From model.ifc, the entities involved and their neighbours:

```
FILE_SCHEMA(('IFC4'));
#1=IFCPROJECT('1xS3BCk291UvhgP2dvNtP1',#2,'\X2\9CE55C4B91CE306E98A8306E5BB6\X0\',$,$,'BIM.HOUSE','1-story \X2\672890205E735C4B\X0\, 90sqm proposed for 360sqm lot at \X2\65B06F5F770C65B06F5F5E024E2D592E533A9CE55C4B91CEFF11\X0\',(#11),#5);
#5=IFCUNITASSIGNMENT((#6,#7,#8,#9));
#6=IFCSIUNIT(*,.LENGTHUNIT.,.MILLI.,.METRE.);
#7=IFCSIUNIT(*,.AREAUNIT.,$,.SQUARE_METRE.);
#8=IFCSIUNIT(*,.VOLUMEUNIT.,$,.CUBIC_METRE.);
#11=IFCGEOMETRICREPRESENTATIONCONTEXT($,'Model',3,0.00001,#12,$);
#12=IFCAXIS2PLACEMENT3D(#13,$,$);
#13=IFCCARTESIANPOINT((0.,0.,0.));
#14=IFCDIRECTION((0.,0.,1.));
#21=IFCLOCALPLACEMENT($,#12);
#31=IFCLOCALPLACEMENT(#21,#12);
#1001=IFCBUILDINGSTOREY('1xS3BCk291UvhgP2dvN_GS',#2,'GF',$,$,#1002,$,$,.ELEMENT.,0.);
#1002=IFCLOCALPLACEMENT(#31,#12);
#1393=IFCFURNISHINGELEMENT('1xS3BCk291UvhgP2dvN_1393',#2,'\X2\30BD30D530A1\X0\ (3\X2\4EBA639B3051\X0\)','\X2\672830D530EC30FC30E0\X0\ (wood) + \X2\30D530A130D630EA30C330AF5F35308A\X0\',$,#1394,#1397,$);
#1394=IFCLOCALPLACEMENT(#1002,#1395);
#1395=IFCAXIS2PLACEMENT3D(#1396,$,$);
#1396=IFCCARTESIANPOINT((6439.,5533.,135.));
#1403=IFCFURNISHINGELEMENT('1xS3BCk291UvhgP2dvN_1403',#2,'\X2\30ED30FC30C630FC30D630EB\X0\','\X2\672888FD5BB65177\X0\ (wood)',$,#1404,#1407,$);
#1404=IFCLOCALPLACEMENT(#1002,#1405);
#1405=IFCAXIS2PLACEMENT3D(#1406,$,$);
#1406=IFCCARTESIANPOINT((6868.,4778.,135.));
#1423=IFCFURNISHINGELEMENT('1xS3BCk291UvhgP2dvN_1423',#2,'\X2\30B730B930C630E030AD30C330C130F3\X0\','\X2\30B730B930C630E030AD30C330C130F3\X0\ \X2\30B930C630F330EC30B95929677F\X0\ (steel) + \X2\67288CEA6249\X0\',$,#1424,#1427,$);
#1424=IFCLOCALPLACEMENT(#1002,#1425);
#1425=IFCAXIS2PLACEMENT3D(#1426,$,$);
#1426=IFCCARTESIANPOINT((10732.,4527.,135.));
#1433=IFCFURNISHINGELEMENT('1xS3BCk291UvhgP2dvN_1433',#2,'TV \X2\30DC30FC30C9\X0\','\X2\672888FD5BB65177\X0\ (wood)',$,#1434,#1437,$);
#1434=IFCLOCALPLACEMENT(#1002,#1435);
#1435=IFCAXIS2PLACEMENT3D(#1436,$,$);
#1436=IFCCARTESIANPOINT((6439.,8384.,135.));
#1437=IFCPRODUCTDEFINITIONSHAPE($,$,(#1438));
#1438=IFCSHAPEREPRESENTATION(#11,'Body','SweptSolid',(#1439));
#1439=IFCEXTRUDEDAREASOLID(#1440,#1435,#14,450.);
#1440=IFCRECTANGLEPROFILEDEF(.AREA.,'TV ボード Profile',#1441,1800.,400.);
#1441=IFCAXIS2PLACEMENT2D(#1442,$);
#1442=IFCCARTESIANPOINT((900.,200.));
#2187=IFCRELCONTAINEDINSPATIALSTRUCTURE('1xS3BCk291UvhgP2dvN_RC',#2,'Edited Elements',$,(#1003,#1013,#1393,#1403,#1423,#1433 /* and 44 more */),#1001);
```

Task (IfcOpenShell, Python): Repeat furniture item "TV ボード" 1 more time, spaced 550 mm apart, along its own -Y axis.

```python
import ifcopenshell
import ifcopenshell.api.geometry
import ifcopenshell.api.root
import ifcopenshell.util.element
import ifcopenshell.util.placement

model = ifcopenshell.open("model.ifc")


def reuse_history(source, copy):
    """copy_class also copies each property set's owner history, people and application; keep the originals."""
    for rel in copy.IsDefinedBy:
        if rel.is_a("IfcRelDefinesByProperties") and (history := rel.RelatingPropertyDefinition.OwnerHistory):
            rel.RelatingPropertyDefinition.OwnerHistory = source.OwnerHistory
            ifcopenshell.util.element.remove_deep2(model, history)


source = model.by_guid("1xS3BCk291UvhgP2dvN_1433")
base = ifcopenshell.util.placement.get_local_placement(source.ObjectPlacement)
step = -base[:3, 1] * 550.0

for i in range(1, 2):
    copy = ifcopenshell.api.root.copy_class(model, product=source)
    copy.Representation = ifcopenshell.util.element.copy_deep(
        model, source.Representation, exclude=["IfcGeometricRepresentationContext", "IfcRepresentationMap"]
    )
    reuse_history(source, copy)
    matrix = base.copy()
    matrix[:3, 3] += i * step
    print("added at", matrix[:3, 3].round(3) + 0.0)
    ifcopenshell.api.geometry.edit_object_placement(model, product=copy, matrix=matrix, is_si=False)

model.write("model_edited.ifc")
```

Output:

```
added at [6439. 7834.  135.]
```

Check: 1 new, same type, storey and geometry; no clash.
